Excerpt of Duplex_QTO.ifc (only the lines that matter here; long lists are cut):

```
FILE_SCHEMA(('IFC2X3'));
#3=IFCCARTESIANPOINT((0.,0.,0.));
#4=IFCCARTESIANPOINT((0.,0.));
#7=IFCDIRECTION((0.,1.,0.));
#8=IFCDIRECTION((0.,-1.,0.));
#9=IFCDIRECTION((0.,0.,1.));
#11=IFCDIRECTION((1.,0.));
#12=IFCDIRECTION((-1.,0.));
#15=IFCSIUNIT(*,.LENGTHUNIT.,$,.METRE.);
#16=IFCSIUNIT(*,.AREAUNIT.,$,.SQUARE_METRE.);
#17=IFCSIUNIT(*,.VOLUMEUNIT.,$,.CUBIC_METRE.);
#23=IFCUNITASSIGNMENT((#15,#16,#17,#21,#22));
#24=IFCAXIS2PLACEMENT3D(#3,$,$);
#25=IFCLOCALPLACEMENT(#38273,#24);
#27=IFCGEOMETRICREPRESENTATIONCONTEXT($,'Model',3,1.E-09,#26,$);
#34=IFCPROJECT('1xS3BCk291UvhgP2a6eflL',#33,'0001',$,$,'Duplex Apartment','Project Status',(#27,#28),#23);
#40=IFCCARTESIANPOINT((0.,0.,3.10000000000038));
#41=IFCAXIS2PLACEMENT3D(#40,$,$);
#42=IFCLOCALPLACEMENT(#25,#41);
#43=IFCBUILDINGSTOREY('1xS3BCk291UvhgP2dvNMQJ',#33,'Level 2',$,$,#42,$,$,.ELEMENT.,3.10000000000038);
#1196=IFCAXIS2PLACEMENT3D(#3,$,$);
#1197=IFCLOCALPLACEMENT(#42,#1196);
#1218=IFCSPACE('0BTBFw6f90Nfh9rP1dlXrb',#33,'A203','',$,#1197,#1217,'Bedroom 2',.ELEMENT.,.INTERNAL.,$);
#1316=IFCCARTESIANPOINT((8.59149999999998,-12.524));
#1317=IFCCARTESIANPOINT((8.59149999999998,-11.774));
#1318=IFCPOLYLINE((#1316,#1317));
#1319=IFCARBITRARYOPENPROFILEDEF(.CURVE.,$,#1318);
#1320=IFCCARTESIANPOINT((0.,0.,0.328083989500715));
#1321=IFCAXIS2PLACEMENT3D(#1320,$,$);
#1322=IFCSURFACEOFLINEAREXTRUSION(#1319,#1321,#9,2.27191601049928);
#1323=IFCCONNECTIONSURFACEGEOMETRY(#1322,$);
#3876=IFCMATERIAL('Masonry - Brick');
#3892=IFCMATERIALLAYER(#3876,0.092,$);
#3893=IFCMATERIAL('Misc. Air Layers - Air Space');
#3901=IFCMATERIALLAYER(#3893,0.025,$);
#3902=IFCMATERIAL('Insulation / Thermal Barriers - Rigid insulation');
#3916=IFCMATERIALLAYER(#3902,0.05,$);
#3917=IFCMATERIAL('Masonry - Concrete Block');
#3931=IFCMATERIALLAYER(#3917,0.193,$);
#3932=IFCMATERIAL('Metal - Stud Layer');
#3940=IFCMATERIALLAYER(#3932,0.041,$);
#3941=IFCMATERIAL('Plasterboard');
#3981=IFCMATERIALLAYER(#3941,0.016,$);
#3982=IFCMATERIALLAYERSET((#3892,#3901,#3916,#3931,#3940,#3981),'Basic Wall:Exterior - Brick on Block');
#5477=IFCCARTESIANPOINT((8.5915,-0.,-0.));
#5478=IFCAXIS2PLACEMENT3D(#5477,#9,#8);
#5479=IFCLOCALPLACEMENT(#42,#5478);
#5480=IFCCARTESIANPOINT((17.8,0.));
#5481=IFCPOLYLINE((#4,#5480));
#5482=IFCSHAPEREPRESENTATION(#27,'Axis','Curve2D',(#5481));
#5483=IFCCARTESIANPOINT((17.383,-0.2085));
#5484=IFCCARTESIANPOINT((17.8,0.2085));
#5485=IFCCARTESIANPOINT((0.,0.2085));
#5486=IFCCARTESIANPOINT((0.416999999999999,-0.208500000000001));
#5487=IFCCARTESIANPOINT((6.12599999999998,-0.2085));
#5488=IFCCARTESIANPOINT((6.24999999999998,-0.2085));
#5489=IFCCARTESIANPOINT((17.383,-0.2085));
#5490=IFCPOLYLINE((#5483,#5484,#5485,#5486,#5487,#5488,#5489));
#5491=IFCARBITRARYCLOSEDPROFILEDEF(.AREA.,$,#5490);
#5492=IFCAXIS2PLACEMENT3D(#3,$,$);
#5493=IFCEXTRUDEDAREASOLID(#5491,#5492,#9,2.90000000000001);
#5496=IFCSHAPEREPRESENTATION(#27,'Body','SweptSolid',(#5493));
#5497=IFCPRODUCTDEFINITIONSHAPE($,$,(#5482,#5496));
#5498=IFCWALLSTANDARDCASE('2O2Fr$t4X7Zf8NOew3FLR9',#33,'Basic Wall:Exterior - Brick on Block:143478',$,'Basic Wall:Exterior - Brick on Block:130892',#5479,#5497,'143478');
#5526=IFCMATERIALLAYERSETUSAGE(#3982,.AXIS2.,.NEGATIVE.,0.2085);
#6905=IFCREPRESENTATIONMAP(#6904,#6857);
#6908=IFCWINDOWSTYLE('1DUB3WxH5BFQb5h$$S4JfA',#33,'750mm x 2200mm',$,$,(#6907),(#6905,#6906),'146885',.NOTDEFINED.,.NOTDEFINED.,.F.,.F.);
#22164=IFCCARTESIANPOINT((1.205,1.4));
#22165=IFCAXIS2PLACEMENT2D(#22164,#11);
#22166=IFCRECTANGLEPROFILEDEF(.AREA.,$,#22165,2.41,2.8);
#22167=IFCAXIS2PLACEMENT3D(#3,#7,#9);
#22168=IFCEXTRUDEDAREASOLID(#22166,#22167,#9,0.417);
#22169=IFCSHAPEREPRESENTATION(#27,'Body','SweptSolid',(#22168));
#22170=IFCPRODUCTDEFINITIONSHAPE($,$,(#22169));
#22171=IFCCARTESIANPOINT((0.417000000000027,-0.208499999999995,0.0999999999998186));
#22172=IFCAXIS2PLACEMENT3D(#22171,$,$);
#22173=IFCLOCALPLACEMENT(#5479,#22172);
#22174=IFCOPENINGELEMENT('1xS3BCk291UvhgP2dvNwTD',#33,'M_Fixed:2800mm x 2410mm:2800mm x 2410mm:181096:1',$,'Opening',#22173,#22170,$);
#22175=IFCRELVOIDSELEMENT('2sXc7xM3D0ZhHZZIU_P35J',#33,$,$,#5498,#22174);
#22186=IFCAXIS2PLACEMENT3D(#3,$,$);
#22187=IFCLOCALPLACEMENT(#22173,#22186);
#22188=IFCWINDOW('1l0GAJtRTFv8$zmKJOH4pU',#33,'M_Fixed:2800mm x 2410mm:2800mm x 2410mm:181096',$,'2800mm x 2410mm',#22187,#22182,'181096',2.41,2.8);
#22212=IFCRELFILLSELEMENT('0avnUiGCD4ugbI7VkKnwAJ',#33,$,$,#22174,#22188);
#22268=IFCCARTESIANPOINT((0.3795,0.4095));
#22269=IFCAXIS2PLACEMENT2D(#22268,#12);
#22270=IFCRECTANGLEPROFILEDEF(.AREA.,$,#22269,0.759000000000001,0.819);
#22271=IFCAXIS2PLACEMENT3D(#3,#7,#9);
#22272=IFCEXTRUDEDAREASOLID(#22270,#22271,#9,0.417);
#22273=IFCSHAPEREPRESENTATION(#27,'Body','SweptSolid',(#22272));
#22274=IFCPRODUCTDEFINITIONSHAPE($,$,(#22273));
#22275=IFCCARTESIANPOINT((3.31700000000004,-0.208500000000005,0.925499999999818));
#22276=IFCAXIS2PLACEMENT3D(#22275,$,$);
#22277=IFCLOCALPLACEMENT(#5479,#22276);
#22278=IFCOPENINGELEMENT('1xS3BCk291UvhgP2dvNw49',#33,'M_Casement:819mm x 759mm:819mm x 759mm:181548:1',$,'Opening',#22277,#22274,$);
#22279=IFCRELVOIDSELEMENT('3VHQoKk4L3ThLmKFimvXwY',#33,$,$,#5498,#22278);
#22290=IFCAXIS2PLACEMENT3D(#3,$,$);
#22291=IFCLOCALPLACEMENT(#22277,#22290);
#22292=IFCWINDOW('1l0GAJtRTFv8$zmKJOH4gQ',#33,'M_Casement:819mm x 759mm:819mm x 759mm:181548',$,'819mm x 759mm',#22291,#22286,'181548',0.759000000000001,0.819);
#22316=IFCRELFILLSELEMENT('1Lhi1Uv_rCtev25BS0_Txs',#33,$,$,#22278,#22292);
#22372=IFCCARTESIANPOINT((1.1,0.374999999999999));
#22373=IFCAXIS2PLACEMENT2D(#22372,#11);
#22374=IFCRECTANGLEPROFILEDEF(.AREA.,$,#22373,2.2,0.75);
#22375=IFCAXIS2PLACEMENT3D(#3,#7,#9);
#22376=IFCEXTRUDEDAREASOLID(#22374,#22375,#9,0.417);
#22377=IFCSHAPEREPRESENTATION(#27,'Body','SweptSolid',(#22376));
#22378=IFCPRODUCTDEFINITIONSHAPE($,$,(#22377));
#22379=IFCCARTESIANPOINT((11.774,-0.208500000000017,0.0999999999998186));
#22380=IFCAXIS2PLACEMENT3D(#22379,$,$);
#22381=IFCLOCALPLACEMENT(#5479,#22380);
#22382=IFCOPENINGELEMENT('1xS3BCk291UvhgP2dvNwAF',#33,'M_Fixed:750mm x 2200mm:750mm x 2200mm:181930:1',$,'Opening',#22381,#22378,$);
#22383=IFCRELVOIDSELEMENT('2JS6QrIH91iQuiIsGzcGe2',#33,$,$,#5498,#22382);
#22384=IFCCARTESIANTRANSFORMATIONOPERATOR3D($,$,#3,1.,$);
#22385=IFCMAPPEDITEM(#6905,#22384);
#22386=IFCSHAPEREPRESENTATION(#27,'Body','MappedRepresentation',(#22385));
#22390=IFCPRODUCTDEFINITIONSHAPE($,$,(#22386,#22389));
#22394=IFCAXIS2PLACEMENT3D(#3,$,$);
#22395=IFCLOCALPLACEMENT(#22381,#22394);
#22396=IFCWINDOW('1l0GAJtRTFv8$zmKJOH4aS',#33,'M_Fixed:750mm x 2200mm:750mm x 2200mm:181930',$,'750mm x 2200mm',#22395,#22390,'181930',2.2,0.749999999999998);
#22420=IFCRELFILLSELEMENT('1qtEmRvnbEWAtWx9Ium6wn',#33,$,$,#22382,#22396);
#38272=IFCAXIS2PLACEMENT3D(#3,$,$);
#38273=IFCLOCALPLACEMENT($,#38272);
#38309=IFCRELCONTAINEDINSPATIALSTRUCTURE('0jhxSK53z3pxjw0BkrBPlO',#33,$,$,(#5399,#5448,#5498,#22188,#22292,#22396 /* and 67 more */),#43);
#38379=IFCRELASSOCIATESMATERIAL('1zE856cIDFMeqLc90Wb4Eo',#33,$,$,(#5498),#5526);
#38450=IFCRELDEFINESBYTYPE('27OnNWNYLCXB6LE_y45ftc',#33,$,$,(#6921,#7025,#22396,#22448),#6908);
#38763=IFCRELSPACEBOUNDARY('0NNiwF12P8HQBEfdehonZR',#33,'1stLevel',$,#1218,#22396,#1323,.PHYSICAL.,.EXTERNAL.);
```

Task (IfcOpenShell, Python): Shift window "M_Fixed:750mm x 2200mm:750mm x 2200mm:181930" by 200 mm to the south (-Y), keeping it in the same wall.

```python
import numpy as np
import ifcopenshell
import ifcopenshell.api.geometry
import ifcopenshell.util.placement

model = ifcopenshell.open("Duplex_QTO.ifc")

window = model.by_guid("1l0GAJtRTFv8$zmKJOH4aS")
opening = window.FillsVoids[0].RelatingOpeningElement
wall = opening.VoidsElements[0].RelatingBuildingElement

wall_matrix = ifcopenshell.util.placement.get_local_placement(wall.ObjectPlacement)
shift = wall_matrix[:3, 0] * 0.2
before = ifcopenshell.util.placement.get_local_placement(window.ObjectPlacement)[:3, 3].copy()

# The window is placed relative to its opening, so it follows when the opening moves.
matrix = ifcopenshell.util.placement.get_local_placement(opening.ObjectPlacement)
matrix[:3, 3] += shift
ifcopenshell.api.geometry.edit_object_placement(
    model, product=opening, matrix=matrix, is_si=False, should_transform_children=True
)

# Space boundary surfaces are stored in each space's coordinates; move them too.
for rel in window.ProvidesBoundaries:
    if not rel.ConnectionGeometry:
        continue
    surface = rel.ConnectionGeometry.SurfaceOnRelatingElement
    space_matrix = ifcopenshell.util.placement.get_local_placement(rel.RelatingSpace.ObjectPlacement)
    point = np.array(surface.Position.Location.Coordinates) + space_matrix[:3, :3].T @ shift
    surface.Position = model.createIfcAxis2Placement3D(
        model.createIfcCartesianPoint(point.tolist()), surface.Position.Axis, surface.Position.RefDirection
    )

after = ifcopenshell.util.placement.get_local_placement(window.ObjectPlacement)[:3, 3]
print("window moved by", (after - before).round(3) + 0.0)

model.write("Duplex_QTO_v2.ifc")
```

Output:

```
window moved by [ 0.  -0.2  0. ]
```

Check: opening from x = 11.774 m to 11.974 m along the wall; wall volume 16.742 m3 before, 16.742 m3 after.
